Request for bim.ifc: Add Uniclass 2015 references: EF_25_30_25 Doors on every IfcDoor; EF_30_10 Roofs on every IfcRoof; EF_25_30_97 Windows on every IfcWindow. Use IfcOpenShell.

First a look at what the model holds.

```python
import ifcopenshell

model = ifcopenshell.open("bim.ifc")
print(model.schema)
print("classifications:", [c.Name for c in model.by_type("IfcClassification")])
for ifc_class in ("IfcDoor", "IfcRoof", "IfcStair", "IfcWall", "IfcWindow"):
    print(ifc_class, len(model.by_type(ifc_class)))
```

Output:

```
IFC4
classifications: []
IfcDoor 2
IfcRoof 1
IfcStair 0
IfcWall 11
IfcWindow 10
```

```python
import ifcopenshell
import ifcopenshell.api.classification

model = ifcopenshell.open("bim.ifc")

system = ifcopenshell.api.classification.add_classification(model, classification="Uniclass 2015")

codes = {
    "IfcDoor": ("EF_25_30_25", "Doors"),
    "IfcRoof": ("EF_30_10", "Roofs"),
    "IfcWindow": ("EF_25_30_97", "Windows"),
}
for ifc_class, (code, name) in codes.items():
    products = model.by_type(ifc_class)
    ifcopenshell.api.classification.add_reference(
        model, products=products, classification=system, identification=code, name=name
    )
    print(code, len(products))

model.write("bim_updated.ifc")
```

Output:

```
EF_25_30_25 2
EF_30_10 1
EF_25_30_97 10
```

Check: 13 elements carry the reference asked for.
